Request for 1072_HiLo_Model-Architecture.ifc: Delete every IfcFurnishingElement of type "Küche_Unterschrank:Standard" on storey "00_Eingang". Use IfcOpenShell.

First a look at what the model holds.

```python
import ifcopenshell
import ifcopenshell.util.element

model = ifcopenshell.open("1072_HiLo_Model-Architecture.ifc")
print(model.schema)
storey = next(s for s in model.by_type("IfcBuildingStorey") if s.Name == "00_Eingang")
furniture = [e for e in ifcopenshell.util.element.get_decomposition(storey) if e.is_a("IfcFurnishingElement")]
seen = {}
for e in furniture:
    element_type = ifcopenshell.util.element.get_type(e)
    name = element_type.Name if element_type not in (None, e) else None
    seen[name] = seen.get(name, 0) + 1
for name, count in sorted(seen.items(), key=str):
    print(count, "x", name)
```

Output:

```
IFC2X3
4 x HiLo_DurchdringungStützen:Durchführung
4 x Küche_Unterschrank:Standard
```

```python
import ifcopenshell
import ifcopenshell.api.root
import ifcopenshell.util.element

model = ifcopenshell.open("1072_HiLo_Model-Architecture.ifc")

storey = next(s for s in model.by_type("IfcBuildingStorey") if s.Name == "00_Eingang")
furniture = [e for e in ifcopenshell.util.element.get_decomposition(storey) if e.is_a("IfcFurnishingElement")]
targets = [e for e in furniture if (t := ifcopenshell.util.element.get_type(e)) not in (None, e) and t.Name == "Küche_Unterschrank:Standard"]

for e in targets:
    ifcopenshell.api.root.remove_product(model, product=e)
print(len(targets), "removed")

model.write("1072_HiLo_Model-Architecture_edited.ifc")
```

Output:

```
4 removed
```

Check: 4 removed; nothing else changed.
